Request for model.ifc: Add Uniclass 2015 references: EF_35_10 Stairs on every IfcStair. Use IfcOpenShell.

First a look at what the model holds.

```python
import ifcopenshell

model = ifcopenshell.open("model.ifc")
print(model.schema)
print("classifications:", [c.Name for c in model.by_type("IfcClassification")])
for ifc_class in ("IfcDoor", "IfcRoof", "IfcStair", "IfcWall", "IfcWindow"):
    print(ifc_class, len(model.by_type(ifc_class)))
```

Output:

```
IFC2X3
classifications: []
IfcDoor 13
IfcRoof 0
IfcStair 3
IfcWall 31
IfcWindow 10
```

```python
import ifcopenshell
import ifcopenshell.api.classification

model = ifcopenshell.open("model.ifc")

# IFC2X3 requires Source and Edition and has no link from the project to the system.
system = model.create_entity("IfcClassification", Source="NBS", Edition="2015", Name="Uniclass 2015")

codes = {
    "IfcStair": ("EF_35_10", "Stairs"),
}
for ifc_class, (code, name) in codes.items():
    products = model.by_type(ifc_class)
    ifcopenshell.api.classification.add_reference(
        model, products=products, classification=system, identification=code, name=name
    )
    print(code, len(products))

model.write("model_edited.ifc")
```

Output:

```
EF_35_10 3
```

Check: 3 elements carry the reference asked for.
